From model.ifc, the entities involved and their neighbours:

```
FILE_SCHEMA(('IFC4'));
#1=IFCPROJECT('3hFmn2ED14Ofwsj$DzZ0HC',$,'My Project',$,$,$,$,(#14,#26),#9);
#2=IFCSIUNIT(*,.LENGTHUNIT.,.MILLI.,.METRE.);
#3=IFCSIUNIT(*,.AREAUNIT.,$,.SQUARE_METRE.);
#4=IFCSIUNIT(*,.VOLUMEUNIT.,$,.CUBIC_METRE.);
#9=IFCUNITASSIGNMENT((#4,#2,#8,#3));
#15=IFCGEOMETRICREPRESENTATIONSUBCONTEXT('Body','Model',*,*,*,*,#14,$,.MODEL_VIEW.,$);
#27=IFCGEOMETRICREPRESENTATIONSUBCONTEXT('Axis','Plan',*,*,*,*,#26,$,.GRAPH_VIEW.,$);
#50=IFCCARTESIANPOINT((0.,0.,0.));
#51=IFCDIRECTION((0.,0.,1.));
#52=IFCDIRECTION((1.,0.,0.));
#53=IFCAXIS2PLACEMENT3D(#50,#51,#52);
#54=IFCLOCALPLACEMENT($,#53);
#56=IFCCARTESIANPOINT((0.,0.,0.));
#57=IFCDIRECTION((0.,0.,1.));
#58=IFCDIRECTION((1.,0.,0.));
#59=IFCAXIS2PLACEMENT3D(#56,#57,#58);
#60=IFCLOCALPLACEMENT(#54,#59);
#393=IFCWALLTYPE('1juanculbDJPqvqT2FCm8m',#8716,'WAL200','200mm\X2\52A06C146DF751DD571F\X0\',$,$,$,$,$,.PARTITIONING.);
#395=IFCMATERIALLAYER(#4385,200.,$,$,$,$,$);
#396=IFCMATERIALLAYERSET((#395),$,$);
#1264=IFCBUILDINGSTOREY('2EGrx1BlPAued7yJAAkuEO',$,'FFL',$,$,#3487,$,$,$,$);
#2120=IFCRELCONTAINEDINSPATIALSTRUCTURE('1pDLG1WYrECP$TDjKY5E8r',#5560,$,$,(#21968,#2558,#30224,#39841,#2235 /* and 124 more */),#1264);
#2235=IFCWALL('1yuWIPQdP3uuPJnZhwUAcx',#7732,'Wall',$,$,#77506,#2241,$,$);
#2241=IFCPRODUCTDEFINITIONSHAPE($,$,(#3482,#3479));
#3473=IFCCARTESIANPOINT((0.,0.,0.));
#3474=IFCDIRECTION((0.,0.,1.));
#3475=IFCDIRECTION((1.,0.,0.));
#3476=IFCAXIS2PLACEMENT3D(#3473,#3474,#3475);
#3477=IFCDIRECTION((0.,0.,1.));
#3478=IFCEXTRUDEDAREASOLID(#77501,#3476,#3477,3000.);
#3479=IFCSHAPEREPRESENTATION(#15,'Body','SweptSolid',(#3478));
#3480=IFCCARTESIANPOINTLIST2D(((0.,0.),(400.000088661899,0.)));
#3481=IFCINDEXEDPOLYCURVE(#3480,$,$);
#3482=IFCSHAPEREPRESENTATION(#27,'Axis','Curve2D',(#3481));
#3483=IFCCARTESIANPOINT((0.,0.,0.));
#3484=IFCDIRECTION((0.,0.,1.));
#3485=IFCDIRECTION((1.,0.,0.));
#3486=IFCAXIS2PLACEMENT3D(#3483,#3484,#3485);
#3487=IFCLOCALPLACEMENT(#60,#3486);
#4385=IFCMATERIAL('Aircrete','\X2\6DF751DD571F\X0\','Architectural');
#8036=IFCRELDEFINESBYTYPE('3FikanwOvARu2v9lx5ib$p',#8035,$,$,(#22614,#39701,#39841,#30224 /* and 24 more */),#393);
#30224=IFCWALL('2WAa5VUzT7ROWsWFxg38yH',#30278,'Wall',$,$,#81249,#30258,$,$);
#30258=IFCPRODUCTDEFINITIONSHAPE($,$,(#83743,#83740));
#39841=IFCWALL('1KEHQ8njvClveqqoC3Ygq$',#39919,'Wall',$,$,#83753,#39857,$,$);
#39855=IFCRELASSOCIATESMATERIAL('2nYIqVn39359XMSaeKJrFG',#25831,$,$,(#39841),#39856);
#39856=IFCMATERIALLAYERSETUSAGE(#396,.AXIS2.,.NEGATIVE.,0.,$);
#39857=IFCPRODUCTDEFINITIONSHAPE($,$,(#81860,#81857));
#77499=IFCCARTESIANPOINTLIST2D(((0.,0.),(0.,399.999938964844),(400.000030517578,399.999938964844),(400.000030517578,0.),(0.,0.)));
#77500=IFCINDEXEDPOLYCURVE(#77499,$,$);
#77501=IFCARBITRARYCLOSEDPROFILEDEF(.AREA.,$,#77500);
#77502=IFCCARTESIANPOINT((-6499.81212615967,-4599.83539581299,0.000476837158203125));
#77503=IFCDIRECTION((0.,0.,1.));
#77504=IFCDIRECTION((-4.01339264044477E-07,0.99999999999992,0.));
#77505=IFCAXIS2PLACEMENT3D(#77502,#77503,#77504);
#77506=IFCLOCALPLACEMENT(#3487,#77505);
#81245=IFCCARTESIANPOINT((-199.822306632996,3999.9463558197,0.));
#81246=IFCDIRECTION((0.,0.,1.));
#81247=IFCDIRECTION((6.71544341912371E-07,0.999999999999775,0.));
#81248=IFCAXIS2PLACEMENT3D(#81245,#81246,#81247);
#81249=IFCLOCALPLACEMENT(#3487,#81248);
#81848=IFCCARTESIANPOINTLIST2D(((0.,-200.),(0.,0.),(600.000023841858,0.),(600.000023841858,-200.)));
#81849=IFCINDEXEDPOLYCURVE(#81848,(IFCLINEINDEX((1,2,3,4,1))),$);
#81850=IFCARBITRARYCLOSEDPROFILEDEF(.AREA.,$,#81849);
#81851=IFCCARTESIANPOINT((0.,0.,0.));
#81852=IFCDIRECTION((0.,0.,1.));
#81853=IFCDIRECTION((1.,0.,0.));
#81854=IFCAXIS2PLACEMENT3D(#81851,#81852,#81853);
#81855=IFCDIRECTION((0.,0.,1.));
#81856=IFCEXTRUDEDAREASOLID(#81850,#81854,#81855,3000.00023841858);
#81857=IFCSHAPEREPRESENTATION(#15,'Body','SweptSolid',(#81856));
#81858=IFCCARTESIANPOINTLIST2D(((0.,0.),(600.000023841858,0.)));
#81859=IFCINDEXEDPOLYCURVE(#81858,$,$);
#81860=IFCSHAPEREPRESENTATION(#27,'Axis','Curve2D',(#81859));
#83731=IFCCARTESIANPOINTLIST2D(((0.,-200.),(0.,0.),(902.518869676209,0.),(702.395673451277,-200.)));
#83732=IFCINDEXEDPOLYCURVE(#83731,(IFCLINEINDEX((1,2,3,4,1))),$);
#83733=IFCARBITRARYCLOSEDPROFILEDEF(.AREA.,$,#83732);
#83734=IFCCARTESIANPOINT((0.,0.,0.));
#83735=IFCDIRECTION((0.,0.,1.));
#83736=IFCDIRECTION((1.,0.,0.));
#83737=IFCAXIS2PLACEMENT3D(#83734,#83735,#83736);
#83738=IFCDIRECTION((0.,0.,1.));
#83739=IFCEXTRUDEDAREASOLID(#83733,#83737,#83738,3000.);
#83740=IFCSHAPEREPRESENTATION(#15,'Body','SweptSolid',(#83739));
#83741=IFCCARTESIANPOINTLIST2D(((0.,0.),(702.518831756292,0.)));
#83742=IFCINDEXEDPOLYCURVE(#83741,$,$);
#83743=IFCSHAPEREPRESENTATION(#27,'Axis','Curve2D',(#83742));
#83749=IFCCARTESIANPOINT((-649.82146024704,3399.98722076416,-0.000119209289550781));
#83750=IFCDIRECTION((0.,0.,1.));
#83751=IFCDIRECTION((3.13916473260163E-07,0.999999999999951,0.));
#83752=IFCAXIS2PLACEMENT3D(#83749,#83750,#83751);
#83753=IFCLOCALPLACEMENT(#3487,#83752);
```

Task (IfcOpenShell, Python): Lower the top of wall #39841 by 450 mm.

```python
import ifcopenshell
import ifcopenshell.geom
import ifcopenshell.util.representation
import ifcopenshell.util.shape

model = ifcopenshell.open("model.ifc")
settings = ifcopenshell.geom.settings()


def volume(element):
    """Net volume in cubic metres, openings subtracted."""
    shape = ifcopenshell.geom.create_shape(settings, element)
    return ifcopenshell.util.shape.get_volume(shape.geometry)


wall = model.by_id(39841)
before = volume(wall)

body = ifcopenshell.util.representation.get_representation(wall, "Model", "Body")
solid = body.Items[0]
old_height = solid.Depth
solid.Depth -= 450.0
after = volume(wall)

print(f"height {old_height:g} -> {solid.Depth:g}, volume {before:.3f} -> {after:.3f} m3")

model.write("model_rev.ifc")
```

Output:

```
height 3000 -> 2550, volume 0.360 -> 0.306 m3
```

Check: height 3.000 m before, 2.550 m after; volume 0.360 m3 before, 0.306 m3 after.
